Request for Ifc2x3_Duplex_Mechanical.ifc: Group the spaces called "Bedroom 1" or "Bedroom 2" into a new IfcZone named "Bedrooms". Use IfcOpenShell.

First a look at what the model holds.

```python
import ifcopenshell

model = ifcopenshell.open("Ifc2x3_Duplex_Mechanical.ifc")
print(model.schema)
seen = {}
for space in model.by_type("IfcSpace"):
    seen[space.LongName] = seen.get(space.LongName, 0) + 1
for name, count in sorted(seen.items(), key=str):
    print(count, "x", name)
print("zones:", [z.Name for z in model.by_type("IfcZone")][:20])
```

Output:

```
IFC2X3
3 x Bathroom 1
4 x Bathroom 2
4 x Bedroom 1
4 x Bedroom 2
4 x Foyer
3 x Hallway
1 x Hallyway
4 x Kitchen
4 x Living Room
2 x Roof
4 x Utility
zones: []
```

```python
import ifcopenshell
import ifcopenshell.api.group
import ifcopenshell.api.root

model = ifcopenshell.open("Ifc2x3_Duplex_Mechanical.ifc")

names = {"Bedroom 1", "Bedroom 2"}
spaces = [s for s in model.by_type("IfcSpace") if s.LongName in names]

zone = ifcopenshell.api.root.create_entity(model, ifc_class="IfcZone", name="Bedrooms")
ifcopenshell.api.group.assign_group(model, products=spaces, group=zone)
print(len(spaces), "spaces in", zone.Name)

model.write("Ifc2x3_Duplex_Mechanical_edited.ifc")
```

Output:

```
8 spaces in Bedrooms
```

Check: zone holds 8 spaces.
